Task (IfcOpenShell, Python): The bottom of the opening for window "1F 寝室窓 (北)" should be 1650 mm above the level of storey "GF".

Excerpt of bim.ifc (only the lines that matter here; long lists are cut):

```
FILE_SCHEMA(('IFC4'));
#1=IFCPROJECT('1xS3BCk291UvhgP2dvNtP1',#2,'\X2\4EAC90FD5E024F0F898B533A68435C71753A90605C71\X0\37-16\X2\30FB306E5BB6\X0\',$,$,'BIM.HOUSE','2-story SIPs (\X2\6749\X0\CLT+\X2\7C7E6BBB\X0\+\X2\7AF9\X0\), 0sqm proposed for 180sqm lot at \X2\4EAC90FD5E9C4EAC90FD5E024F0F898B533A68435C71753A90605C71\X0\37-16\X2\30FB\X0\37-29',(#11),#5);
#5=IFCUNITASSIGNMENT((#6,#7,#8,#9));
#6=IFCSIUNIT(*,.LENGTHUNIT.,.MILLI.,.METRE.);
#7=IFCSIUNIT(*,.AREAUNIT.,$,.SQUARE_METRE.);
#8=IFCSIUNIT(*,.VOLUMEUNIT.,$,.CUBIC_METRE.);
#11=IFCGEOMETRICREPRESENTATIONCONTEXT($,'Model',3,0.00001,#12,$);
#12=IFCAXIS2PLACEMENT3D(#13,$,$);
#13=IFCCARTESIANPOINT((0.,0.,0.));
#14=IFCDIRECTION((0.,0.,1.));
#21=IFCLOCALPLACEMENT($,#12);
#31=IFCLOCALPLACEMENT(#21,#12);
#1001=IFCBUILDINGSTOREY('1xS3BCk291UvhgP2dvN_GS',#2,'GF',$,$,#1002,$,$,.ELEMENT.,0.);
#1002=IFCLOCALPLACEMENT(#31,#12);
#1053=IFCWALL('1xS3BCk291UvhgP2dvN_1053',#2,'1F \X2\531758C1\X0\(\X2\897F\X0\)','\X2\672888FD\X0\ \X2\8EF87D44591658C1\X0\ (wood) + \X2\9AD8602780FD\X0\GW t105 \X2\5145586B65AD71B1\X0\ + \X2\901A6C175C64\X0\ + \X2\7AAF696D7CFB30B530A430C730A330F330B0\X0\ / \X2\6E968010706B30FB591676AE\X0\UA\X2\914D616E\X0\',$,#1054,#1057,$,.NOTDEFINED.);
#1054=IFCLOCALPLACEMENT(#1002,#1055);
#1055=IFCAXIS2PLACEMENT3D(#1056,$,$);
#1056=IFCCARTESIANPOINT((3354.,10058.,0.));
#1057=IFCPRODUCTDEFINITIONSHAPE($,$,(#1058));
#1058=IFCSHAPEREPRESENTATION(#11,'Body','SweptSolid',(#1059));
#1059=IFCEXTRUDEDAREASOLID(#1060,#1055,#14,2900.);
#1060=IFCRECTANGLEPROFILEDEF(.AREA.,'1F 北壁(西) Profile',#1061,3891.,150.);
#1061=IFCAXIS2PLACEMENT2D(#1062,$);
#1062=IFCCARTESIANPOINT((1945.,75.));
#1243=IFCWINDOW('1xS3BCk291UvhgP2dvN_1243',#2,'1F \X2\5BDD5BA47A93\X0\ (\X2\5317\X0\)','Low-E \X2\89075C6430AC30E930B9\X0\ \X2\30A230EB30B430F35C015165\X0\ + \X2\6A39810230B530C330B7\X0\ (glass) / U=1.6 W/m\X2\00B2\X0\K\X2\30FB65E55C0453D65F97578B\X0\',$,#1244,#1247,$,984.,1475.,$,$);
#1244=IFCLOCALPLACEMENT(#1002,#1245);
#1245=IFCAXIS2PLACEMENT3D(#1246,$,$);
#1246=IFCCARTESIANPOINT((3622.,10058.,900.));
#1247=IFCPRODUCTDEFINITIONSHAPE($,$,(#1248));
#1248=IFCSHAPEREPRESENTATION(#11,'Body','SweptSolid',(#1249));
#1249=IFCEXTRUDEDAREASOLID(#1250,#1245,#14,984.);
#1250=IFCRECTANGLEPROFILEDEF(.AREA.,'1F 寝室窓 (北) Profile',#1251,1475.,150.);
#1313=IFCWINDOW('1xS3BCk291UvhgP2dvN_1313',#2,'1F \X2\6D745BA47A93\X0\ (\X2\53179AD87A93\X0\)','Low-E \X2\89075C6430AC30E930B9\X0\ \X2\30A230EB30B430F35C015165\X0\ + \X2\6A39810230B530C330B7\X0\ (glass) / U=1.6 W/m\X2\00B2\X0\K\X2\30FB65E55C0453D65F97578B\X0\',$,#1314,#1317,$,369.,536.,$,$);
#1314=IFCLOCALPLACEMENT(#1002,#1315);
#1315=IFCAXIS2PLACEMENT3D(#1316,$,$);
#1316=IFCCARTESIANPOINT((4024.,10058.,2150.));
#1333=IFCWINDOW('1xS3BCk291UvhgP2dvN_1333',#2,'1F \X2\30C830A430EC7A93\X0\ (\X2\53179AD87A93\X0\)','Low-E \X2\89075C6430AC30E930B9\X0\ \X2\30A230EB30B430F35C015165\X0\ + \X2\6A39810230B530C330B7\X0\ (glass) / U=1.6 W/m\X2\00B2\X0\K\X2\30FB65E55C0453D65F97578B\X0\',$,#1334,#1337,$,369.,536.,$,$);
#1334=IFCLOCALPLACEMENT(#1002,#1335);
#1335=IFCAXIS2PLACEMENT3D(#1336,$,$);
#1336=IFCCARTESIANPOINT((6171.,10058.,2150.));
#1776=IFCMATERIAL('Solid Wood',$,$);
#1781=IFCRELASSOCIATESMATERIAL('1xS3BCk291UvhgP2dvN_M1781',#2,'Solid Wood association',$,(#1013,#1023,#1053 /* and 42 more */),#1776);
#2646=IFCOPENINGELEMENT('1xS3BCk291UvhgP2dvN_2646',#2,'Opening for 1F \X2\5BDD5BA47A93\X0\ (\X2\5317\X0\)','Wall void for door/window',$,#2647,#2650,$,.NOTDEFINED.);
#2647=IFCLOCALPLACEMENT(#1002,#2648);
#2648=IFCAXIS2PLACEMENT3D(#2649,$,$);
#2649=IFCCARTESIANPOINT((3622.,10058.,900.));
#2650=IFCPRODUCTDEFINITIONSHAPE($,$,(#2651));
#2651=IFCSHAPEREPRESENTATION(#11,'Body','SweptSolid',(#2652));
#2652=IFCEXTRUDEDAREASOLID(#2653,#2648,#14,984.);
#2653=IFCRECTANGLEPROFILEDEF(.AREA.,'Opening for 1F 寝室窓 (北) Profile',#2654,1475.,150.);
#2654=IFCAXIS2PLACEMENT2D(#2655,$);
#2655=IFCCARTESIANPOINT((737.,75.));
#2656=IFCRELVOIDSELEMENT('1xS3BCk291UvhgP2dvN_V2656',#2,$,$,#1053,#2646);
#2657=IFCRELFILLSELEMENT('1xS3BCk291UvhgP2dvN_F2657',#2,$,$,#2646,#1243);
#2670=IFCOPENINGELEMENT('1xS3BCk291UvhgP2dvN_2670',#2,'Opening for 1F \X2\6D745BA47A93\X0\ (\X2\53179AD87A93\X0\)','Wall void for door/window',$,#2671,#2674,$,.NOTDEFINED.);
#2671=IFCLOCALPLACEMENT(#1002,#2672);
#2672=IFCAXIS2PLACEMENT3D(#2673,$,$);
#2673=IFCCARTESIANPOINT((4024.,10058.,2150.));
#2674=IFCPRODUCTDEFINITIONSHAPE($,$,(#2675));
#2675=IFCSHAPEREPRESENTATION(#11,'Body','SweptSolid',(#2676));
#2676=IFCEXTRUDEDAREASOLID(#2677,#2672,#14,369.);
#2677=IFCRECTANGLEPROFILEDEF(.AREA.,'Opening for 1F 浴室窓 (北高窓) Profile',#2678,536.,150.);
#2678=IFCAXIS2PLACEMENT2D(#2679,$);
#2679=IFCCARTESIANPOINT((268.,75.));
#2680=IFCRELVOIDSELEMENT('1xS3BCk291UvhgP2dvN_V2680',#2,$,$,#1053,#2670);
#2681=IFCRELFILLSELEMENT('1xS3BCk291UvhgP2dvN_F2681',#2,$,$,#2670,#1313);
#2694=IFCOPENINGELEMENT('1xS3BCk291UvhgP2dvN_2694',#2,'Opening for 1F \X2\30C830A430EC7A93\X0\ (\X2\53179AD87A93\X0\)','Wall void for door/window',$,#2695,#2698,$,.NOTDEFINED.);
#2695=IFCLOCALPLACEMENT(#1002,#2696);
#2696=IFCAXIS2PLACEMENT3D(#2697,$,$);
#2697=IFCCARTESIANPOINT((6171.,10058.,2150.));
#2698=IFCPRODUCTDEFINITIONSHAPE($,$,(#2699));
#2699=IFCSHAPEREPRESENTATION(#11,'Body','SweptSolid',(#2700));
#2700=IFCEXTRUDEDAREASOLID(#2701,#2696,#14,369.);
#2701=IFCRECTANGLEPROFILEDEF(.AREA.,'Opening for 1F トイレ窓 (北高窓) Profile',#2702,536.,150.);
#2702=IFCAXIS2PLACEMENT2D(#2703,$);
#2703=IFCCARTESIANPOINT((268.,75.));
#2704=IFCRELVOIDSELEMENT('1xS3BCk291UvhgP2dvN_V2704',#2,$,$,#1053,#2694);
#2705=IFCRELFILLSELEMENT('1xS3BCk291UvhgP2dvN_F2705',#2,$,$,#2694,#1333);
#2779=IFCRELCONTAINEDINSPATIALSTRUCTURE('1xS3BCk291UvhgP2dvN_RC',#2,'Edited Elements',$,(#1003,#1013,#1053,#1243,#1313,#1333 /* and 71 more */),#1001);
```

```python
import numpy as np
import ifcopenshell
import ifcopenshell.api.geometry
import ifcopenshell.geom
import ifcopenshell.util.element
import ifcopenshell.util.placement
import ifcopenshell.util.shape
import ifcopenshell.util.unit

model = ifcopenshell.open("bim.ifc")
unit_scale = ifcopenshell.util.unit.calculate_unit_scale(model)

window = model.by_guid("1xS3BCk291UvhgP2dvN_1243")
opening = window.FillsVoids[0].RelatingOpeningElement
storey = ifcopenshell.util.element.get_container(window, ifc_class="IfcBuildingStorey")
level = ifcopenshell.util.placement.get_local_placement(storey.ObjectPlacement)[2, 3]

# The opening's origin need not be at the sill, so measure its lowest point.
shape = ifcopenshell.geom.create_shape(ifcopenshell.geom.settings(), opening)
bottom = ifcopenshell.util.shape.get_shape_bottom_elevation(shape, shape.geometry) / unit_scale
dz = level + 1650.0 - bottom

shift = np.array([0.0, 0.0, dz])
# The window is not placed relative to its opening, so move both.
for product in (opening, window):
    matrix = ifcopenshell.util.placement.get_local_placement(product.ObjectPlacement)
    matrix[:3, 3] += shift
    ifcopenshell.api.geometry.edit_object_placement(model, product=product, matrix=matrix, is_si=False)

print(f"moved by {dz * unit_scale:+.3f} m")

model.write("bim-out.ifc")
```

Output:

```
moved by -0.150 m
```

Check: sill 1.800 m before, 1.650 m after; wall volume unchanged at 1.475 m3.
